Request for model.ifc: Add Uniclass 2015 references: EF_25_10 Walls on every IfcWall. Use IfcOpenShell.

First a look at what the model holds.

```python
import ifcopenshell

model = ifcopenshell.open("model.ifc")
print(model.schema)
print("classifications:", [c.Name for c in model.by_type("IfcClassification")])
for ifc_class in ("IfcDoor", "IfcRoof", "IfcStair", "IfcWall", "IfcWindow"):
    print(ifc_class, len(model.by_type(ifc_class)))
```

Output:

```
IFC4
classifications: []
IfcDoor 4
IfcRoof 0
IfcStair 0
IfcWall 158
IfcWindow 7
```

```python
import ifcopenshell
import ifcopenshell.api.classification

model = ifcopenshell.open("model.ifc")

system = ifcopenshell.api.classification.add_classification(model, classification="Uniclass 2015")

codes = {
    "IfcWall": ("EF_25_10", "Walls"),
}
for ifc_class, (code, name) in codes.items():
    products = model.by_type(ifc_class)
    ifcopenshell.api.classification.add_reference(
        model, products=products, classification=system, identification=code, name=name
    )
    print(code, len(products))

model.write("model_rev.ifc")
```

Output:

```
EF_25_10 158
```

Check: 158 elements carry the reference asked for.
